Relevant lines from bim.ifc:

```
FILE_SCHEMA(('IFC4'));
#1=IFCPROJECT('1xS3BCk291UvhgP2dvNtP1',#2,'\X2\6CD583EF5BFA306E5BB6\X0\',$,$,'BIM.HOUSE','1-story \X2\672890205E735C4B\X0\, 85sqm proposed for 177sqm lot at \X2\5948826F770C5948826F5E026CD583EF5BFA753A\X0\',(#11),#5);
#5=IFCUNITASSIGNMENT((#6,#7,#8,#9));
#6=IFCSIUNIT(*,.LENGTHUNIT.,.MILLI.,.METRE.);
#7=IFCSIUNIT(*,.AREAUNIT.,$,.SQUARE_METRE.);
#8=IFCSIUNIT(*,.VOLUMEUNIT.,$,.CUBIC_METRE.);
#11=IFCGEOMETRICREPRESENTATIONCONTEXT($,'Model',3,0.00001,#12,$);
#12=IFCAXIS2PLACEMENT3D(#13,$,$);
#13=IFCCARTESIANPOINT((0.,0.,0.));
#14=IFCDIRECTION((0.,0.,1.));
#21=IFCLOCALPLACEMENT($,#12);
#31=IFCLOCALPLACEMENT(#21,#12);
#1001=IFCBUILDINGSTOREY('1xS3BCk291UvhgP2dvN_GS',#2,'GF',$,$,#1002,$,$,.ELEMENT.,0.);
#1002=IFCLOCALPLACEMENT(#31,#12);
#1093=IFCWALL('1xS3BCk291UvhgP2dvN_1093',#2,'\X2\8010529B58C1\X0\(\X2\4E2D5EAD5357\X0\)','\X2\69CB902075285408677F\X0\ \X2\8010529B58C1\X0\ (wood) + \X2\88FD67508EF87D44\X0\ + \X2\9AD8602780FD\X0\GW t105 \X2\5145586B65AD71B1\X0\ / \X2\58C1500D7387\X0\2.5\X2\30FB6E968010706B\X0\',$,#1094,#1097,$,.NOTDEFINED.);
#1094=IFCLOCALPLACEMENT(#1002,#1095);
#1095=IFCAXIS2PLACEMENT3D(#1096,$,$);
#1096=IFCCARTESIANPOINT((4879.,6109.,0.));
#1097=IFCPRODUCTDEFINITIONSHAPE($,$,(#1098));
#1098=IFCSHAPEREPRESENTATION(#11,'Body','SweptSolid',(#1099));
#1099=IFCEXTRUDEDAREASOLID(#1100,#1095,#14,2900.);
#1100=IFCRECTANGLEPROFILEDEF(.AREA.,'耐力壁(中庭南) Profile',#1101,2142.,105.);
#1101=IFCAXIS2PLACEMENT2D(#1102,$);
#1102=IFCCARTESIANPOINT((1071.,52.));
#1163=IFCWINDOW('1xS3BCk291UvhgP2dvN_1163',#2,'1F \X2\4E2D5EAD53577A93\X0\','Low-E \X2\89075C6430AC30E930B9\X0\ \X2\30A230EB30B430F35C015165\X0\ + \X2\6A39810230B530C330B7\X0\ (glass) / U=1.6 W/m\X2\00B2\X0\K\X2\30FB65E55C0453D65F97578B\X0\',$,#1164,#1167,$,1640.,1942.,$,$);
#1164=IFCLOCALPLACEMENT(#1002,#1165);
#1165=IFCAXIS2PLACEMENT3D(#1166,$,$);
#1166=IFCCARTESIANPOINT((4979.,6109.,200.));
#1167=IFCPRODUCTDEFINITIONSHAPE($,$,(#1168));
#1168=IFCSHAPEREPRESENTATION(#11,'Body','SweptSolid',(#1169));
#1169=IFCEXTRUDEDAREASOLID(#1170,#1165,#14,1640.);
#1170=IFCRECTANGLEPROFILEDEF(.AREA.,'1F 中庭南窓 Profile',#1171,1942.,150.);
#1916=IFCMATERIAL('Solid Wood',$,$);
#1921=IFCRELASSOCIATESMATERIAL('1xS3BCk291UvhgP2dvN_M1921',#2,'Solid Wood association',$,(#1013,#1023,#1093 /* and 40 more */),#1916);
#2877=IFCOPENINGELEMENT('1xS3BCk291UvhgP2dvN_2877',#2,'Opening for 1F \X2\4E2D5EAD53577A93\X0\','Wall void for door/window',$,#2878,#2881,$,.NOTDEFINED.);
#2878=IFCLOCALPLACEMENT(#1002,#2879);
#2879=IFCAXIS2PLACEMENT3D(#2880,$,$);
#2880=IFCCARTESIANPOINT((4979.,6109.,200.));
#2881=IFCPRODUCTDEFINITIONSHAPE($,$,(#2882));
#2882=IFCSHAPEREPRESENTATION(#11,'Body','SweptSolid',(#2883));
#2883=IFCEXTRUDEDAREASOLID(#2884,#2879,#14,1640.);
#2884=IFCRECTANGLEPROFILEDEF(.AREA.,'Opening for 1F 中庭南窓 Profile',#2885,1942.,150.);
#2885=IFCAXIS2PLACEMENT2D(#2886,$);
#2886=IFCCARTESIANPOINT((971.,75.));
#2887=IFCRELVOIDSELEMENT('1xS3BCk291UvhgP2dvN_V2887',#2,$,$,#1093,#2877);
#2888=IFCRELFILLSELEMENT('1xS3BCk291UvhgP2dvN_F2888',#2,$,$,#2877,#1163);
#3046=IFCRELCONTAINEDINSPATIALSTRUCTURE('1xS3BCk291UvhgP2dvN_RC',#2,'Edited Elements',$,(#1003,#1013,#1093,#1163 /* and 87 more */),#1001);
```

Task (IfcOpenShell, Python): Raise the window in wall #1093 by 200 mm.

```python
import numpy as np
import ifcopenshell
import ifcopenshell.api.geometry
import ifcopenshell.util.placement
import ifcopenshell.util.unit

model = ifcopenshell.open("bim.ifc")
unit_scale = ifcopenshell.util.unit.calculate_unit_scale(model)

window = model.by_guid("1xS3BCk291UvhgP2dvN_1163")
opening = window.FillsVoids[0].RelatingOpeningElement
dz = 200.0

shift = np.array([0.0, 0.0, dz])
# The window is not placed relative to its opening, so move both.
for product in (opening, window):
    matrix = ifcopenshell.util.placement.get_local_placement(product.ObjectPlacement)
    matrix[:3, 3] += shift
    ifcopenshell.api.geometry.edit_object_placement(model, product=product, matrix=matrix, is_si=False)

print(f"moved by {dz * unit_scale:+.3f} m")

model.write("bim_updated.ifc")
```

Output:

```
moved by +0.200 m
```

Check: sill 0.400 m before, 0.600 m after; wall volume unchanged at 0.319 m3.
